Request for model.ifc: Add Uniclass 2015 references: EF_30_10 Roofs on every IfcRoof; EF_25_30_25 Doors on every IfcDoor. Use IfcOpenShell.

First a look at what the model holds.

```python
import ifcopenshell

model = ifcopenshell.open("model.ifc")
print(model.schema)
print("classifications:", [c.Name for c in model.by_type("IfcClassification")])
for ifc_class in ("IfcDoor", "IfcRoof", "IfcStair", "IfcWall", "IfcWindow"):
    print(ifc_class, len(model.by_type(ifc_class)))
```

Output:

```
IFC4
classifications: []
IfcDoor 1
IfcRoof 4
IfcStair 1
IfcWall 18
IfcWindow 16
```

```python
import ifcopenshell
import ifcopenshell.api.classification

model = ifcopenshell.open("model.ifc")

system = ifcopenshell.api.classification.add_classification(model, classification="Uniclass 2015")

codes = {
    "IfcRoof": ("EF_30_10", "Roofs"),
    "IfcDoor": ("EF_25_30_25", "Doors"),
}
for ifc_class, (code, name) in codes.items():
    products = model.by_type(ifc_class)
    ifcopenshell.api.classification.add_reference(
        model, products=products, classification=system, identification=code, name=name
    )
    print(code, len(products))

model.write("model-out.ifc")
```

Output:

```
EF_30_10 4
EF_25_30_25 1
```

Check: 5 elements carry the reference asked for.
